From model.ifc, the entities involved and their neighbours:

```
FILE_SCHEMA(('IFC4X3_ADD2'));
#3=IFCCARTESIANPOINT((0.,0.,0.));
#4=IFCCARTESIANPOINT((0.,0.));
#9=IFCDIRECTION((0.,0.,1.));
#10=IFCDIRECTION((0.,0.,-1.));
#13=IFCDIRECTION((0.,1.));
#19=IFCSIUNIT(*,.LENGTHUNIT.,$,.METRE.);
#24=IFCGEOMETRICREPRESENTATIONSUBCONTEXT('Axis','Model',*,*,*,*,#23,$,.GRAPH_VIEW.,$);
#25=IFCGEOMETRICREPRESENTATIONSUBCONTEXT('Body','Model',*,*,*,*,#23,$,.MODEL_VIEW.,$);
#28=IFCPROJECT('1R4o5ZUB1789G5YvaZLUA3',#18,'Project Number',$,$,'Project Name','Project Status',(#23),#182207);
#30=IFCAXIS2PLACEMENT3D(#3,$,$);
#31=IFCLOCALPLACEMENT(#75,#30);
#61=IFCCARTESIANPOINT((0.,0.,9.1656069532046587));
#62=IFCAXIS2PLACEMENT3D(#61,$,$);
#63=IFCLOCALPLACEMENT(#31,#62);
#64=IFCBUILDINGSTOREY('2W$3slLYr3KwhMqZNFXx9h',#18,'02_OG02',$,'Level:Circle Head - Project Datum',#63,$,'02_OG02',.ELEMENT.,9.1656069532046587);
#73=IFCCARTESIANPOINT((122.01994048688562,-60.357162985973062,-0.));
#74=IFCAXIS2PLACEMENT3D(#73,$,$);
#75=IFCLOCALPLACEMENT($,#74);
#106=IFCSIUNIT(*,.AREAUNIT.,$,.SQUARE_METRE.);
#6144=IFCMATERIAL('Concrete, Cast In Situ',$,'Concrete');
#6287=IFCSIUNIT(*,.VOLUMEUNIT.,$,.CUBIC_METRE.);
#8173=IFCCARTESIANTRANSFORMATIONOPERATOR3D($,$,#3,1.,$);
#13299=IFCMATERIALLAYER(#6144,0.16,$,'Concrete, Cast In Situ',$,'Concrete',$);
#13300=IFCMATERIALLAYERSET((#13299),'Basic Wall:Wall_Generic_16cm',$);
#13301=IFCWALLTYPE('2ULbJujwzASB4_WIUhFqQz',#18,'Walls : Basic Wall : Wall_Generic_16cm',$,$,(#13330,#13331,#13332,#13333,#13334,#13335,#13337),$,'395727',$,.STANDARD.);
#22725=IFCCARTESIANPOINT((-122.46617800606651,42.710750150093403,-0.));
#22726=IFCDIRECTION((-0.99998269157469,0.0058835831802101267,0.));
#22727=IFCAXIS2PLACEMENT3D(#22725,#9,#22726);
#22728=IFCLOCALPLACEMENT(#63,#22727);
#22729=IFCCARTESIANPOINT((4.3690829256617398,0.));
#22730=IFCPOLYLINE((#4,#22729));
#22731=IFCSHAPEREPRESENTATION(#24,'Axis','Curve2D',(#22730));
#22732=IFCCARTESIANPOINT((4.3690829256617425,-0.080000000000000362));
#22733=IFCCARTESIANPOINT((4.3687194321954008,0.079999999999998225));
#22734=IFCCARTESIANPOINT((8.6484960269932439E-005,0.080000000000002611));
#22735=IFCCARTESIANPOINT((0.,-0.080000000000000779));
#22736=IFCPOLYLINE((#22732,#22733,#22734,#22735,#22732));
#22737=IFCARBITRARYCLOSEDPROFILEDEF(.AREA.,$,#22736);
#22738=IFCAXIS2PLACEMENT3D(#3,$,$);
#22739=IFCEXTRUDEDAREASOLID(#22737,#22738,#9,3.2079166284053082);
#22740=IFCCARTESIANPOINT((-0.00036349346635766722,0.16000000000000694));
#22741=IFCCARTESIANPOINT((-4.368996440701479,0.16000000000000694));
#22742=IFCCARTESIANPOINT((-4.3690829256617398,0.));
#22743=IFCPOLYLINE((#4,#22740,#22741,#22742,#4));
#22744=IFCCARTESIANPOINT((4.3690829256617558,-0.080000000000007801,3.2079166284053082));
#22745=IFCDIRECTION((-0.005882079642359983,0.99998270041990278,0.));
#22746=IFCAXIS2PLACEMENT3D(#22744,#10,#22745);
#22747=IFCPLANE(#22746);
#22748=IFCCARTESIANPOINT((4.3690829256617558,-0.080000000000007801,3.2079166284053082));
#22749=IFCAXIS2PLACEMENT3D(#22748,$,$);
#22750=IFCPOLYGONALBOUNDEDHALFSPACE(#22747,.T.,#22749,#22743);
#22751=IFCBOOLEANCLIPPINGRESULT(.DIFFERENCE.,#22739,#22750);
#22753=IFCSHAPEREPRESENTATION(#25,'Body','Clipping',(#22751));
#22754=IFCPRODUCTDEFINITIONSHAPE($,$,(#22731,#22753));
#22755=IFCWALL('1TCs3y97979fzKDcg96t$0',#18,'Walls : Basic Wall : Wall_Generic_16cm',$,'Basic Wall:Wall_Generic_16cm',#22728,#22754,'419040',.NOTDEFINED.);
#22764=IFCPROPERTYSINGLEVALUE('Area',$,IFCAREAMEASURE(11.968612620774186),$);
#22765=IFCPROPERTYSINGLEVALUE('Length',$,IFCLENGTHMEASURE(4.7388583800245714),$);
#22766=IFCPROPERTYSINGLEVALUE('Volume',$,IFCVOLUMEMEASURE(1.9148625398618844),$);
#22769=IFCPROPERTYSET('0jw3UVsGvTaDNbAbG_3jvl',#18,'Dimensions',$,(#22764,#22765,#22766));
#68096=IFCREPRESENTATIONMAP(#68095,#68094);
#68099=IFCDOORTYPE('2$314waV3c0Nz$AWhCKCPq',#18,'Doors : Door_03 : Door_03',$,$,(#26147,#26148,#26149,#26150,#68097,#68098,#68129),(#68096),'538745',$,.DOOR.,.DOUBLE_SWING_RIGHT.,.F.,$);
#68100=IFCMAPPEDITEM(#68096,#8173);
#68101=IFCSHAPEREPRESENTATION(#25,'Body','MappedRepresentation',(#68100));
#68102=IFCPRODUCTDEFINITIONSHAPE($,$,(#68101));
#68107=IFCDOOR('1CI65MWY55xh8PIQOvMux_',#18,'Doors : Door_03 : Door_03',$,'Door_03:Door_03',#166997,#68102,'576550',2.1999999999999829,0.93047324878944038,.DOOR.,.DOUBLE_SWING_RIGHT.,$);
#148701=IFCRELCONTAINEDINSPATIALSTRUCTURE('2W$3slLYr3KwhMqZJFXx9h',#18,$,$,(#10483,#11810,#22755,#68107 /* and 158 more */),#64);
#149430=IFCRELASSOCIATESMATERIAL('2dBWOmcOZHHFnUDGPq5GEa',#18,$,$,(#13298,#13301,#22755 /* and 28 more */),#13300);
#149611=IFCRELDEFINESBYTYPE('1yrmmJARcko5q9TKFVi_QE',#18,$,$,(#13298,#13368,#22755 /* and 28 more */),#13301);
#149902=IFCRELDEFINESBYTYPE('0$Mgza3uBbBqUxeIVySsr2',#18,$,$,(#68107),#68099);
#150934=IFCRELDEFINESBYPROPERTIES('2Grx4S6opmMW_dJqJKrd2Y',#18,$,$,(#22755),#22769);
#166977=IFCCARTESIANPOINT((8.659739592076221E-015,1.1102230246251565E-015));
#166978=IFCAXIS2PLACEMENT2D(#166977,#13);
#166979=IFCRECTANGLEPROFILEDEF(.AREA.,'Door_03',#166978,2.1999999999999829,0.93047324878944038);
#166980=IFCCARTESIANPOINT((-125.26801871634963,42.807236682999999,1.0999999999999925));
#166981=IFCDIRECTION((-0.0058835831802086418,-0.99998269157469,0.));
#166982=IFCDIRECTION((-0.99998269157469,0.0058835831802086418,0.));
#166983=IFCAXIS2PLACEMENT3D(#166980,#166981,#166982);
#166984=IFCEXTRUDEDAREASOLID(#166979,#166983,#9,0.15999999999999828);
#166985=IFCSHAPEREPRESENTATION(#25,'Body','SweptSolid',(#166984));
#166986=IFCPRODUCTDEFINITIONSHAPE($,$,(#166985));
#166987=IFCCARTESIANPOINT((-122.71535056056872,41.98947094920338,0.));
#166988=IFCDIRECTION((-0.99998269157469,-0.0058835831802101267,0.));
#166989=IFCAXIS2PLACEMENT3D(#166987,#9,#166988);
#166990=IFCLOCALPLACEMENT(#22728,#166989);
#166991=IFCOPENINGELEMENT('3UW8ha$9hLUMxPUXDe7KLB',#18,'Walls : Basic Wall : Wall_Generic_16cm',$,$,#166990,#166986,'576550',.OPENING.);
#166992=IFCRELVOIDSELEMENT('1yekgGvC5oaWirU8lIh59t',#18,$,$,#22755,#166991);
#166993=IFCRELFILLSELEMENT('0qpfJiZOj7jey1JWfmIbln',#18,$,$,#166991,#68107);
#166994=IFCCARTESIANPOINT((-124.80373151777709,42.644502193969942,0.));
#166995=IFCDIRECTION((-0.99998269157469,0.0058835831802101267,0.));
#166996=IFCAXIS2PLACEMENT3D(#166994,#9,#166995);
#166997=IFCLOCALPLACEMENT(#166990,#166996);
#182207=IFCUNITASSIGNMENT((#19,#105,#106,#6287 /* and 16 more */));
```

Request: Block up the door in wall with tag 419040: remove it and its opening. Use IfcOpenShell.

```python
import ifcopenshell
import ifcopenshell.api.feature
import ifcopenshell.api.pset
import ifcopenshell.api.root
import ifcopenshell.geom
import ifcopenshell.util.element
import ifcopenshell.util.shape
import ifcopenshell.util.unit

model = ifcopenshell.open("model.ifc")
area_scale = ifcopenshell.util.unit.calculate_unit_scale(model, "AREAUNIT")
volume_scale = ifcopenshell.util.unit.calculate_unit_scale(model, "VOLUMEUNIT")
settings = ifcopenshell.geom.settings()


def volume(element):
    """Net volume in cubic metres, openings subtracted."""
    shape = ifcopenshell.geom.create_shape(settings, element)
    return ifcopenshell.util.shape.get_volume(shape.geometry)


door = model.by_guid("1CI65MWY55xh8PIQOvMux_")
opening = door.FillsVoids[0].RelatingOpeningElement
wall = opening.VoidsElements[0].RelatingBuildingElement
before = volume(wall)

ifcopenshell.api.root.remove_product(model, product=door)
ifcopenshell.api.feature.remove_feature(model, feature=opening)

after = volume(wall)
thickness = 0.16  # wall thickness in metres

# Update the wall's stored quantities.
pset = model.by_id(ifcopenshell.util.element.get_pset(wall, "Dimensions", should_inherit=False)["id"])
ifcopenshell.api.pset.edit_pset(model, pset=pset, properties={
    "Area": model.create_entity("IfcAreaMeasure", after / thickness / area_scale),
    "Volume": model.create_entity("IfcVolumeMeasure", after / volume_scale),
})

print(f"wall volume {before:.3f} -> {after:.3f} m3")

model.write("model-out.ifc")
```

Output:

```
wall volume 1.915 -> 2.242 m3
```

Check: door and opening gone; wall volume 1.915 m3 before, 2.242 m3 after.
